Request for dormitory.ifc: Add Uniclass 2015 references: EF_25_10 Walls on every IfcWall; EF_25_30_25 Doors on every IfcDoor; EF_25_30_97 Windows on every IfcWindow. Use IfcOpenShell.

First a look at what the model holds.

```python
import ifcopenshell

model = ifcopenshell.open("dormitory.ifc")
print(model.schema)
print("classifications:", [c.Name for c in model.by_type("IfcClassification")])
for ifc_class in ("IfcDoor", "IfcRoof", "IfcStair", "IfcWall", "IfcWindow"):
    print(ifc_class, len(model.by_type(ifc_class)))
```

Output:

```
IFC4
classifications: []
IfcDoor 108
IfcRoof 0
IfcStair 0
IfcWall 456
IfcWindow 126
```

```python
import ifcopenshell
import ifcopenshell.api.classification

model = ifcopenshell.open("dormitory.ifc")

system = ifcopenshell.api.classification.add_classification(model, classification="Uniclass 2015")

codes = {
    "IfcWall": ("EF_25_10", "Walls"),
    "IfcDoor": ("EF_25_30_25", "Doors"),
    "IfcWindow": ("EF_25_30_97", "Windows"),
}
for ifc_class, (code, name) in codes.items():
    products = model.by_type(ifc_class)
    ifcopenshell.api.classification.add_reference(
        model, products=products, classification=system, identification=code, name=name
    )
    print(code, len(products))

model.write("dormitory_rev.ifc")
```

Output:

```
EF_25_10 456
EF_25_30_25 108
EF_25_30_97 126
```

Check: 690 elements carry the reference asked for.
